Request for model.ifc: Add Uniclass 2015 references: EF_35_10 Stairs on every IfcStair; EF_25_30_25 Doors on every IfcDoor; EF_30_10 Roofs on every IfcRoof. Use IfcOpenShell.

First a look at what the model holds.

```python
import ifcopenshell

model = ifcopenshell.open("model.ifc")
print(model.schema)
print("classifications:", [c.Name for c in model.by_type("IfcClassification")])
for ifc_class in ("IfcDoor", "IfcRoof", "IfcStair", "IfcWall", "IfcWindow"):
    print(ifc_class, len(model.by_type(ifc_class)))
```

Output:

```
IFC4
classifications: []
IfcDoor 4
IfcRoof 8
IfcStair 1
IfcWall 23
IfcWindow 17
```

```python
import ifcopenshell
import ifcopenshell.api.classification

model = ifcopenshell.open("model.ifc")

system = ifcopenshell.api.classification.add_classification(model, classification="Uniclass 2015")

codes = {
    "IfcStair": ("EF_35_10", "Stairs"),
    "IfcDoor": ("EF_25_30_25", "Doors"),
    "IfcRoof": ("EF_30_10", "Roofs"),
}
for ifc_class, (code, name) in codes.items():
    products = model.by_type(ifc_class)
    ifcopenshell.api.classification.add_reference(
        model, products=products, classification=system, identification=code, name=name
    )
    print(code, len(products))

model.write("model-out.ifc")
```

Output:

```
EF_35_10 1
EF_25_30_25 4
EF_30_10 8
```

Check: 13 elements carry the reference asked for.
